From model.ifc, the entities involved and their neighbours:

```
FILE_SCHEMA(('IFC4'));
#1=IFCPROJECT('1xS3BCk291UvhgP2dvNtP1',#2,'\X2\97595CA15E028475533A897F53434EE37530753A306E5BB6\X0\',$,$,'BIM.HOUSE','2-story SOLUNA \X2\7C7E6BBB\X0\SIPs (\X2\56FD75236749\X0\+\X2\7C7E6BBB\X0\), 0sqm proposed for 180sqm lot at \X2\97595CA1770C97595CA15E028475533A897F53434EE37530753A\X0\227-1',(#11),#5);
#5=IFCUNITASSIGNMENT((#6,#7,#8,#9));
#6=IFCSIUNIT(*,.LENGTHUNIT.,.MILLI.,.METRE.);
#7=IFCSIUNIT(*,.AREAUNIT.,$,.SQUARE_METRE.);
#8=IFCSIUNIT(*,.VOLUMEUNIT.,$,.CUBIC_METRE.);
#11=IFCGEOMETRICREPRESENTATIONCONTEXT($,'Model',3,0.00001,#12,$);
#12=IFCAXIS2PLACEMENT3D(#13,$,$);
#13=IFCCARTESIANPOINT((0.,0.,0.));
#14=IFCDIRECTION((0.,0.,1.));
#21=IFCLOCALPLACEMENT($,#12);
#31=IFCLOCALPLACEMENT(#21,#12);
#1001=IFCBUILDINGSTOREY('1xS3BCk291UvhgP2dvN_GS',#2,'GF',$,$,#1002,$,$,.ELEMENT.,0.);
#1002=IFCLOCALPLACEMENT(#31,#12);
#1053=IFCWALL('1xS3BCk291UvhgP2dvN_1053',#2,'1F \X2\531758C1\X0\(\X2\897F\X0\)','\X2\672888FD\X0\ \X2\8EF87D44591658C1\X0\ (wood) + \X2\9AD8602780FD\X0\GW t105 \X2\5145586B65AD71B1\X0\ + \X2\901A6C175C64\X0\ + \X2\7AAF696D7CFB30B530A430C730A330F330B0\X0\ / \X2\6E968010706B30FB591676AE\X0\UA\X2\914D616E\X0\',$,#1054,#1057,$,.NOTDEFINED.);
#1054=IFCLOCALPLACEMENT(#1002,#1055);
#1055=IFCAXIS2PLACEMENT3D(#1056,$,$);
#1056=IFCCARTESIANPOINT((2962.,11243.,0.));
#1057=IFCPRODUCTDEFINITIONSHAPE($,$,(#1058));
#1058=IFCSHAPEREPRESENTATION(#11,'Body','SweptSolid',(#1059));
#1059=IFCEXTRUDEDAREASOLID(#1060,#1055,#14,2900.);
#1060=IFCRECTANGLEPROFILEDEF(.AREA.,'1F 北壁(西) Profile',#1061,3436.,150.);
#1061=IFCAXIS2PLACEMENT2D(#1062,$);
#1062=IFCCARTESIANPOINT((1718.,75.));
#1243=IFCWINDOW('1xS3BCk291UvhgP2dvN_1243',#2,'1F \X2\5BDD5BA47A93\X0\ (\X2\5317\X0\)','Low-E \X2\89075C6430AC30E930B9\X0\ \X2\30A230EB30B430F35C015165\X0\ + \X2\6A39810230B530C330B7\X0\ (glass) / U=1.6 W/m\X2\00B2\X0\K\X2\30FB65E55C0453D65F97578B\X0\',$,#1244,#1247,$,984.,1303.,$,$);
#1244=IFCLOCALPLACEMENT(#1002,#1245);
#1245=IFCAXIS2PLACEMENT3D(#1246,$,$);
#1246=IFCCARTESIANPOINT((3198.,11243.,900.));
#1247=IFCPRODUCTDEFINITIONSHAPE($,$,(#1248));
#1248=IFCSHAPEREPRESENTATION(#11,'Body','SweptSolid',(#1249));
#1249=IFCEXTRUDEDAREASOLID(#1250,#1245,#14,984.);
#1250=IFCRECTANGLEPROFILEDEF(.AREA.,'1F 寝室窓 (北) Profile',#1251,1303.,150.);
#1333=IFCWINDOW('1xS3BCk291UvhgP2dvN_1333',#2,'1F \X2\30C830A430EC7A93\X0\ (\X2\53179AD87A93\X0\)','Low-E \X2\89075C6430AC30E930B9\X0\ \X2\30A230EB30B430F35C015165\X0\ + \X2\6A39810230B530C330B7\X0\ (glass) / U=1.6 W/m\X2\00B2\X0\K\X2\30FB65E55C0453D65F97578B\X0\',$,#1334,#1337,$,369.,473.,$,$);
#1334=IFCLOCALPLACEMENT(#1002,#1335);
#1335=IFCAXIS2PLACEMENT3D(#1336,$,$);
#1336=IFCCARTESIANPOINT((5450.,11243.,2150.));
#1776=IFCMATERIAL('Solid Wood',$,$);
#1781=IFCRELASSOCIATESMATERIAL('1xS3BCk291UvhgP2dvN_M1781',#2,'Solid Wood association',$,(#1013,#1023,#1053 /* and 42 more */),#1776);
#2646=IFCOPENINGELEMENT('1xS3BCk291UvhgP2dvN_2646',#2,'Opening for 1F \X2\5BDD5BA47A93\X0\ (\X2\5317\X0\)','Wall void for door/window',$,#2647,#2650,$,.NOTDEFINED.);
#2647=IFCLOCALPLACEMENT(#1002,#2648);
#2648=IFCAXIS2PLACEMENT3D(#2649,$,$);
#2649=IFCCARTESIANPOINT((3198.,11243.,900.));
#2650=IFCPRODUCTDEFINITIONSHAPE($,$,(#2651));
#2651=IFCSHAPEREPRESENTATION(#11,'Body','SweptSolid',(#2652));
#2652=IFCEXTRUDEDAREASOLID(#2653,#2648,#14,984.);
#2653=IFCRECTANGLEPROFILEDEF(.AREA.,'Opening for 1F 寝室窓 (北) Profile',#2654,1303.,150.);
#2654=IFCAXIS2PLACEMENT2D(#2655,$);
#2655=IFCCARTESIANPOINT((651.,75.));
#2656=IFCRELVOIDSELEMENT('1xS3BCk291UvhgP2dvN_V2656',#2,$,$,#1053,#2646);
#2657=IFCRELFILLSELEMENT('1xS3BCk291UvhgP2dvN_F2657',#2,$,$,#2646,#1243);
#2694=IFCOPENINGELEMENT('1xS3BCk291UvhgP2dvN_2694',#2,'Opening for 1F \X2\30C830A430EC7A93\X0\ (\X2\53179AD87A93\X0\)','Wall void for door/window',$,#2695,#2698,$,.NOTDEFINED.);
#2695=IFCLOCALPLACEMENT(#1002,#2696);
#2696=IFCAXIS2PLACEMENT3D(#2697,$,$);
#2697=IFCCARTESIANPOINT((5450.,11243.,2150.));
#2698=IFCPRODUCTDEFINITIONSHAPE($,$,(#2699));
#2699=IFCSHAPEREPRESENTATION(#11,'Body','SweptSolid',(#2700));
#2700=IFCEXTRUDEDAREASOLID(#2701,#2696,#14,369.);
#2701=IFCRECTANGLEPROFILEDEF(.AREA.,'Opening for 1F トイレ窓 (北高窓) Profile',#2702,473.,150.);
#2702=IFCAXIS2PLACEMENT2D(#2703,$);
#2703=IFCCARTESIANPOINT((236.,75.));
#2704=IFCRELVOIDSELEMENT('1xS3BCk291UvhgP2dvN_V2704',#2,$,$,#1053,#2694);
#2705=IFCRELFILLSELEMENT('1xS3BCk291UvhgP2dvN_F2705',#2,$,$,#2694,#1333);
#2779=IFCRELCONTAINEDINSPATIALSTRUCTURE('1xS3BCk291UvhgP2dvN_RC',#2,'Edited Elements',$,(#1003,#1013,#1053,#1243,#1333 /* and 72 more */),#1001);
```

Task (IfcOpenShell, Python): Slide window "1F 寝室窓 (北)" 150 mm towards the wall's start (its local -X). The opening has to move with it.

```python
import ifcopenshell
import ifcopenshell.api.geometry
import ifcopenshell.util.placement

model = ifcopenshell.open("model.ifc")

window = model.by_guid("1xS3BCk291UvhgP2dvN_1243")
opening = window.FillsVoids[0].RelatingOpeningElement
wall = opening.VoidsElements[0].RelatingBuildingElement

wall_matrix = ifcopenshell.util.placement.get_local_placement(wall.ObjectPlacement)
shift = wall_matrix[:3, 0] * -150.0
before = ifcopenshell.util.placement.get_local_placement(window.ObjectPlacement)[:3, 3].copy()

# The window is not placed relative to its opening, so move both.
for product in (opening, window):
    matrix = ifcopenshell.util.placement.get_local_placement(product.ObjectPlacement)
    matrix[:3, 3] += shift
    ifcopenshell.api.geometry.edit_object_placement(model, product=product, matrix=matrix, is_si=False)

after = ifcopenshell.util.placement.get_local_placement(window.ObjectPlacement)[:3, 3]
print("window moved by", (after - before).round(3) + 0.0)

model.write("model_rev.ifc")
```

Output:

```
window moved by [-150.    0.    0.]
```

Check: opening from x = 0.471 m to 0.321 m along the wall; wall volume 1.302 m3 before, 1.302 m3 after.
